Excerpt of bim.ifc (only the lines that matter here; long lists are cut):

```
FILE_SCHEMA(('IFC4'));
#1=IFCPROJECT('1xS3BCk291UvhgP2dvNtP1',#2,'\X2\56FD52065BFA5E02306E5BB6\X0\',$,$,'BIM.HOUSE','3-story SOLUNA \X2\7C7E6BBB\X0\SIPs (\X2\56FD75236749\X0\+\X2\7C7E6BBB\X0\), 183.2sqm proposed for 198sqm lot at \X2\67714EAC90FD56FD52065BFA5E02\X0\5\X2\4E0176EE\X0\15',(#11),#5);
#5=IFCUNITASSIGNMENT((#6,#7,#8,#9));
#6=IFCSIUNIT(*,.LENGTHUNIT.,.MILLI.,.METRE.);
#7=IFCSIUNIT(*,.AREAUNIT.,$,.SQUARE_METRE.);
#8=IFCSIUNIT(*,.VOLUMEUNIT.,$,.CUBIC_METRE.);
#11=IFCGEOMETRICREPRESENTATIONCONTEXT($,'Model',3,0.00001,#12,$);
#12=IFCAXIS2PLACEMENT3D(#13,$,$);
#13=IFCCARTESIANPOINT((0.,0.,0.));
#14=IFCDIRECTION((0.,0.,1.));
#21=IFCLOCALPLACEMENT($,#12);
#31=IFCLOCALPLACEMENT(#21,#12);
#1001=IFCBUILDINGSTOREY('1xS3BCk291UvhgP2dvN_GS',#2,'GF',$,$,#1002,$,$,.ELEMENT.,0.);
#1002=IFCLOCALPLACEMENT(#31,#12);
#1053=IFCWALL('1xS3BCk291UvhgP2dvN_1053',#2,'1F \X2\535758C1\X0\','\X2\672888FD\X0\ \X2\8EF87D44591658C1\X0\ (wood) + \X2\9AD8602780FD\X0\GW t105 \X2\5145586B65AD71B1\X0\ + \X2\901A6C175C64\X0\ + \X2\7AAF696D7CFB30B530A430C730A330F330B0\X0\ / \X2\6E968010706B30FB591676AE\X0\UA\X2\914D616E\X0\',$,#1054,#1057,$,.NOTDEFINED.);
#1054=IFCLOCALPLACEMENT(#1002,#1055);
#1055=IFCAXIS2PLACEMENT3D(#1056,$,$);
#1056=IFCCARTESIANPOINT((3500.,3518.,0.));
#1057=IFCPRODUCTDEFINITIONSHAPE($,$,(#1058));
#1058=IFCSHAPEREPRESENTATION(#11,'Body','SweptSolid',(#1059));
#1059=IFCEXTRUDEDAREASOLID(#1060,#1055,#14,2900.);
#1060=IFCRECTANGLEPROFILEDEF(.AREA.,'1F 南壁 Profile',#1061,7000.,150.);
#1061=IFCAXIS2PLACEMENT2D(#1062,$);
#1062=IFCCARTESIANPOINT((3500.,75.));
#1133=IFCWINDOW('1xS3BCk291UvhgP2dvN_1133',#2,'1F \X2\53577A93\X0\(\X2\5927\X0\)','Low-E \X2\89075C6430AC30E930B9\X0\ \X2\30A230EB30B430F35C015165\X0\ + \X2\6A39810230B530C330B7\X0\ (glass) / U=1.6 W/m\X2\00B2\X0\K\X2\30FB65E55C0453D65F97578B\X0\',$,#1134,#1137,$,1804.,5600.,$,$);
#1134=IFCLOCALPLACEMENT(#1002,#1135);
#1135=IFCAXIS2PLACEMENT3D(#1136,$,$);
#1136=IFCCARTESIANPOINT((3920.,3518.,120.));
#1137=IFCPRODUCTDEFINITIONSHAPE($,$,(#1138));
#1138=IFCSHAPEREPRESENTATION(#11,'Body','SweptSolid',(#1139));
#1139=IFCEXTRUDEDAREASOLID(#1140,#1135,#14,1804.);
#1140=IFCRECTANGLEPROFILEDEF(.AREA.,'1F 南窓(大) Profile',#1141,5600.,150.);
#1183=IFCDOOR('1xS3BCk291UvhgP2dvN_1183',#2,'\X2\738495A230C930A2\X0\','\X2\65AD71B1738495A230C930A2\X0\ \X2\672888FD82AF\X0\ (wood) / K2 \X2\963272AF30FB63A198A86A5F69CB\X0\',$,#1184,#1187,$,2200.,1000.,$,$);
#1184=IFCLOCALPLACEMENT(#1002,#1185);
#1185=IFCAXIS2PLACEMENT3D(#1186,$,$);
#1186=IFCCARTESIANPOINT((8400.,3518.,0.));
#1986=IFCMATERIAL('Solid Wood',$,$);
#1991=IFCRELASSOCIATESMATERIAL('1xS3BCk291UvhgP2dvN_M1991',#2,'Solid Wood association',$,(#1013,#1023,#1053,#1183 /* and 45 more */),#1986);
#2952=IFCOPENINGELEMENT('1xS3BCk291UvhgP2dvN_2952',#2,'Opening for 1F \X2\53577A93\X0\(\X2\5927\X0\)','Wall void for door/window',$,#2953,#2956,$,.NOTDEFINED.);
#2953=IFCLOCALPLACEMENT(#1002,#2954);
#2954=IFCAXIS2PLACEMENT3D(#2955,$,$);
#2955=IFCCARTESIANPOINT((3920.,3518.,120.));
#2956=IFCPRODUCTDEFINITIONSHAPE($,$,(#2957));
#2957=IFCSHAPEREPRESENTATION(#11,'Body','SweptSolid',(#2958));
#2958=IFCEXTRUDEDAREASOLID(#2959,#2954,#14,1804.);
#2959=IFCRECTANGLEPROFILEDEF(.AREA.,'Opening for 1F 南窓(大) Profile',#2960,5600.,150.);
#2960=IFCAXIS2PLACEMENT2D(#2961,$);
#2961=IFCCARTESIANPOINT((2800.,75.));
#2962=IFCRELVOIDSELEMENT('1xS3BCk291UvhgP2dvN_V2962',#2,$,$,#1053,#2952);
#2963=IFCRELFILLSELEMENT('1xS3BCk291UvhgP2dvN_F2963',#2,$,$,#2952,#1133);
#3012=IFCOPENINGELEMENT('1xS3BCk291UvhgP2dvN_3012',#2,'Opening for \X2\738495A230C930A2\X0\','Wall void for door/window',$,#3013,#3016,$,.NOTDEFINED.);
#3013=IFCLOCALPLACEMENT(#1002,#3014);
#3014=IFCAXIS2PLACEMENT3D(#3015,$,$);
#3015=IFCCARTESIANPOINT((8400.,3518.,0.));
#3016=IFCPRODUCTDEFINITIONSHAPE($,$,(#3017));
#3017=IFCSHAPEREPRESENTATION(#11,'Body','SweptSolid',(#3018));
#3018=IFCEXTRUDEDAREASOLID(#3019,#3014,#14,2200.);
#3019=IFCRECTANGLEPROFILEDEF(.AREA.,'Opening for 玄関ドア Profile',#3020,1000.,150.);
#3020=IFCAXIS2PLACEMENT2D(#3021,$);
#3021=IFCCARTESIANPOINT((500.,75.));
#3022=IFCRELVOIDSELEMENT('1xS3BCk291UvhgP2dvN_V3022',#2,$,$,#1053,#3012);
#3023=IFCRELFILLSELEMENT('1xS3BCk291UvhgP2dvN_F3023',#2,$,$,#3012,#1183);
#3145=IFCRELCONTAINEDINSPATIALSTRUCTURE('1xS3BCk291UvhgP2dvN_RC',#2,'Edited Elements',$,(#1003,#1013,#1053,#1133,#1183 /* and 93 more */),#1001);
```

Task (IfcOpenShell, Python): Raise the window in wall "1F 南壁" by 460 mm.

```python
import numpy as np
import ifcopenshell
import ifcopenshell.api.geometry
import ifcopenshell.util.placement
import ifcopenshell.util.unit

model = ifcopenshell.open("bim.ifc")
unit_scale = ifcopenshell.util.unit.calculate_unit_scale(model)

window = model.by_guid("1xS3BCk291UvhgP2dvN_1133")
opening = window.FillsVoids[0].RelatingOpeningElement
dz = 460.0

shift = np.array([0.0, 0.0, dz])
# The window is not placed relative to its opening, so move both.
for product in (opening, window):
    matrix = ifcopenshell.util.placement.get_local_placement(product.ObjectPlacement)
    matrix[:3, 3] += shift
    ifcopenshell.api.geometry.edit_object_placement(model, product=product, matrix=matrix, is_si=False)

print(f"moved by {dz * unit_scale:+.3f} m")

model.write("bim-out.ifc")
```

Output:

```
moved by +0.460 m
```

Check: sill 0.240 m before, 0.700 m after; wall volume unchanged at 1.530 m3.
